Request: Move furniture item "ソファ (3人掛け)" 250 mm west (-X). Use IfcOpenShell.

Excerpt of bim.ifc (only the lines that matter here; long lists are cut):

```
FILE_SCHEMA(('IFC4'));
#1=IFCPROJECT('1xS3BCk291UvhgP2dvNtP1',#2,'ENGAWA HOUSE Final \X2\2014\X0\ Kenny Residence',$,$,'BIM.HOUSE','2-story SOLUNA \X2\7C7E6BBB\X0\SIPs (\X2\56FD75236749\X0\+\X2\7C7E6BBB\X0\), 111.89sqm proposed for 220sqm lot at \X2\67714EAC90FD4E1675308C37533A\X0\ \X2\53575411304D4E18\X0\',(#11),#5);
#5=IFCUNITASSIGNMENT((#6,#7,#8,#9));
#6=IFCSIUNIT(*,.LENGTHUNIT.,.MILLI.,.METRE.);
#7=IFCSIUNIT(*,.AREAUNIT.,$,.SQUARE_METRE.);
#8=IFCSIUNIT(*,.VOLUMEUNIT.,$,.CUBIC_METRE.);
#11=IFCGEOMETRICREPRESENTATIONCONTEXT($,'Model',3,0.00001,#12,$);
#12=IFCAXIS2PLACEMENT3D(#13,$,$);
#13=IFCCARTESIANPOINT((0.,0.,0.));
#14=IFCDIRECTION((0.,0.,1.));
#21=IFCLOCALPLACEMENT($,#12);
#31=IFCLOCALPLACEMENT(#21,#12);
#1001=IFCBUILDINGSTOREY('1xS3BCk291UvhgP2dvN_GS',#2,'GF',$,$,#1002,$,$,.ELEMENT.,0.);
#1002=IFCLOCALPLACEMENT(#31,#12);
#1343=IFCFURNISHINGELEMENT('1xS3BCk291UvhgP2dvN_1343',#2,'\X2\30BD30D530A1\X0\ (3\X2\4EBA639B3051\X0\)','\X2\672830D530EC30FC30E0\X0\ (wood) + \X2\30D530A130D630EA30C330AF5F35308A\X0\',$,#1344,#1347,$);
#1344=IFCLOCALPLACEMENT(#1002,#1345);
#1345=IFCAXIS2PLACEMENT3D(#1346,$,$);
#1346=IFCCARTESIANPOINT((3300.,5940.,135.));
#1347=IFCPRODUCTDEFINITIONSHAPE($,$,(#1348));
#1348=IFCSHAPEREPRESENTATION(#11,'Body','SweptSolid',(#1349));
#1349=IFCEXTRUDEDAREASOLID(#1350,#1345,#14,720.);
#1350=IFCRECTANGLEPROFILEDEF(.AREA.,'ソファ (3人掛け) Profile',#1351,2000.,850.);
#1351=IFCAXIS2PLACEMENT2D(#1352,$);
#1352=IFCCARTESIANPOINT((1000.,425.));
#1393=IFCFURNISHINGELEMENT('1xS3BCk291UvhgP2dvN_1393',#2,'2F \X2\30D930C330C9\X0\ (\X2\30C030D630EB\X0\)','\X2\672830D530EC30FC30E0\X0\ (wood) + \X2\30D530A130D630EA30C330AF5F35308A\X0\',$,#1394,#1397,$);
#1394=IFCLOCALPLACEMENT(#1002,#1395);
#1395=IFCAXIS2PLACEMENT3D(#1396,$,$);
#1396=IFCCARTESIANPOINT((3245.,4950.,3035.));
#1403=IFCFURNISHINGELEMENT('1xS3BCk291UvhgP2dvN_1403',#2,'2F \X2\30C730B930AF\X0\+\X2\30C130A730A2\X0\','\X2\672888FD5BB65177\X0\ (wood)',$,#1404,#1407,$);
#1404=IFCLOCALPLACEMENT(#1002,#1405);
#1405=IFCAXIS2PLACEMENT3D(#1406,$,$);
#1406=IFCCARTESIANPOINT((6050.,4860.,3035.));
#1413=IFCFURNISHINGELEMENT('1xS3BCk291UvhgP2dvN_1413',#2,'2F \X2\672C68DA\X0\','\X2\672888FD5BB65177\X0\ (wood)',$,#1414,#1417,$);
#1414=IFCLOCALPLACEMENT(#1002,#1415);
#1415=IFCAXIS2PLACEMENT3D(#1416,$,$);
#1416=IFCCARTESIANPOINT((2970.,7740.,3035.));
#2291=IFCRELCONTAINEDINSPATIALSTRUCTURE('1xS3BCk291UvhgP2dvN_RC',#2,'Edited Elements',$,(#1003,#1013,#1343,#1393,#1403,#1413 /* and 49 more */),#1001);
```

```python
import ifcopenshell
import ifcopenshell.api.geometry
import ifcopenshell.util.placement
import ifcopenshell.util.unit

model = ifcopenshell.open("bim.ifc")
unit_scale = ifcopenshell.util.unit.calculate_unit_scale(model)

item = model.by_id(1343)
matrix = ifcopenshell.util.placement.get_local_placement(item.ObjectPlacement)
matrix[0, 3] -= 0.25 / unit_scale
ifcopenshell.api.geometry.edit_object_placement(model, product=item, matrix=matrix, is_si=False)

print(ifcopenshell.util.placement.get_local_placement(item.ObjectPlacement).round(3) + 0.0)

model.write("bim_updated.ifc")
```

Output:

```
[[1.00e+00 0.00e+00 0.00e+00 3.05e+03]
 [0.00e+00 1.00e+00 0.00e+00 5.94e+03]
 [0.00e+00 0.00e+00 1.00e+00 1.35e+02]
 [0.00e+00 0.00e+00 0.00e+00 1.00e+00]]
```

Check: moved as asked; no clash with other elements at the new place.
